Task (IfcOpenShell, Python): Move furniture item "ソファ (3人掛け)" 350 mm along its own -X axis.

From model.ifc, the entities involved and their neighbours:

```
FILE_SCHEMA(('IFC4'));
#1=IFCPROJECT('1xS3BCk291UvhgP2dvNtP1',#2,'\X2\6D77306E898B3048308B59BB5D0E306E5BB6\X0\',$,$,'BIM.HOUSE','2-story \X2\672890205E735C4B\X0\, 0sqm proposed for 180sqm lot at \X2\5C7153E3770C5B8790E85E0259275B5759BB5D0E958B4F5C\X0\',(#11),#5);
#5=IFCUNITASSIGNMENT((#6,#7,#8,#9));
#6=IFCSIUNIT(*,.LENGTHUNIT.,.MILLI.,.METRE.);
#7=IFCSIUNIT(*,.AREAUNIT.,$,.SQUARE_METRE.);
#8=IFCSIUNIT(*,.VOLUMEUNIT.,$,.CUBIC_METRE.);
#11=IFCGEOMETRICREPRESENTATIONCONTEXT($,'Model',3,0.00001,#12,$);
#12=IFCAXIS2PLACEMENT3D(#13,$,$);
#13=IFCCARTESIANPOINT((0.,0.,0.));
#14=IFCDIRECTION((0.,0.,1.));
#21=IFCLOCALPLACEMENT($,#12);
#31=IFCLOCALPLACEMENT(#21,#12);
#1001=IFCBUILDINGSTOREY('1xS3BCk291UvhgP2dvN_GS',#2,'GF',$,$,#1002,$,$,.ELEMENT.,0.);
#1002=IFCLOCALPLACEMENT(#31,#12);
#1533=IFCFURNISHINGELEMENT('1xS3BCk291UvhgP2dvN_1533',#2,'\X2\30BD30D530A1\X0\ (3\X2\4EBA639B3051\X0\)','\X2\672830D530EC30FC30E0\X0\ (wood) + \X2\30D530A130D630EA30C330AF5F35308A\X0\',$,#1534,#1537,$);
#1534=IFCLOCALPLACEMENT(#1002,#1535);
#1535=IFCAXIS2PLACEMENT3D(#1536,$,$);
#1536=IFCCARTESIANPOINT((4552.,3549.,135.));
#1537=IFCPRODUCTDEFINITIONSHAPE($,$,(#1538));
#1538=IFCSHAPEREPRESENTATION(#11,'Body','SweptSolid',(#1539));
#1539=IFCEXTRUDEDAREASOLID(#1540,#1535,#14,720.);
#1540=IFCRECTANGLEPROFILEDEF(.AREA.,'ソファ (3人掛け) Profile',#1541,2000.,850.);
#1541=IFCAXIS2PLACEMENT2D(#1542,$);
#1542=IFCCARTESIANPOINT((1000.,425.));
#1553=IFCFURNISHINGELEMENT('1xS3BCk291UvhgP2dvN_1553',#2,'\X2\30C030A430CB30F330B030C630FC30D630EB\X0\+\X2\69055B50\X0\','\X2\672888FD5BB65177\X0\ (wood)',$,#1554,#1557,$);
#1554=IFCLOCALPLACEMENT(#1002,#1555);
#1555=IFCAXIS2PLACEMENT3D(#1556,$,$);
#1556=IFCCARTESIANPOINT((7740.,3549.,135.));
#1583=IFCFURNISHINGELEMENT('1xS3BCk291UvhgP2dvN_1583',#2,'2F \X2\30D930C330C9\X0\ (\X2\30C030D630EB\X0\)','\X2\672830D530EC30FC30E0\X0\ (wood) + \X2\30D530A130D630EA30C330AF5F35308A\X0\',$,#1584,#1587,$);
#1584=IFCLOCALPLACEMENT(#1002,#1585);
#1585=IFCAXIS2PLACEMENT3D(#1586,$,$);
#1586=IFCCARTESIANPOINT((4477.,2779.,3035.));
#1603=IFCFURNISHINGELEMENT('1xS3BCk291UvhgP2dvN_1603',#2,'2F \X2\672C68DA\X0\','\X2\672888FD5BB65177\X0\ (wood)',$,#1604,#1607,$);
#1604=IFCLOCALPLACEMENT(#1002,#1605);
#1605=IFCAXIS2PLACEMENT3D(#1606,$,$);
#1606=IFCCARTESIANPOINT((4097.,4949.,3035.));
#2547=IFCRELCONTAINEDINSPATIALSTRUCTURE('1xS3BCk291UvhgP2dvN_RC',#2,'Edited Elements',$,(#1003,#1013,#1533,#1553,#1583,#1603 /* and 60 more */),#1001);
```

```python
import ifcopenshell
import ifcopenshell.api.geometry
import ifcopenshell.util.placement
import ifcopenshell.util.unit

model = ifcopenshell.open("model.ifc")
unit_scale = ifcopenshell.util.unit.calculate_unit_scale(model)

item = model.by_id(1533)
matrix = ifcopenshell.util.placement.get_local_placement(item.ObjectPlacement)
matrix[:3, 3] -= matrix[:3, 0] * 0.35 / unit_scale
ifcopenshell.api.geometry.edit_object_placement(model, product=item, matrix=matrix, is_si=False)

print(ifcopenshell.util.placement.get_local_placement(item.ObjectPlacement).round(3) + 0.0)

model.write("model_updated.ifc")
```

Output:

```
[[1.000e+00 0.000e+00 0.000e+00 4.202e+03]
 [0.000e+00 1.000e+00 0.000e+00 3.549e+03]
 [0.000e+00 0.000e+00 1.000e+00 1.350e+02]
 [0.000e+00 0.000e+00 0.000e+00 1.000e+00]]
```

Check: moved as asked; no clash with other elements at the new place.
